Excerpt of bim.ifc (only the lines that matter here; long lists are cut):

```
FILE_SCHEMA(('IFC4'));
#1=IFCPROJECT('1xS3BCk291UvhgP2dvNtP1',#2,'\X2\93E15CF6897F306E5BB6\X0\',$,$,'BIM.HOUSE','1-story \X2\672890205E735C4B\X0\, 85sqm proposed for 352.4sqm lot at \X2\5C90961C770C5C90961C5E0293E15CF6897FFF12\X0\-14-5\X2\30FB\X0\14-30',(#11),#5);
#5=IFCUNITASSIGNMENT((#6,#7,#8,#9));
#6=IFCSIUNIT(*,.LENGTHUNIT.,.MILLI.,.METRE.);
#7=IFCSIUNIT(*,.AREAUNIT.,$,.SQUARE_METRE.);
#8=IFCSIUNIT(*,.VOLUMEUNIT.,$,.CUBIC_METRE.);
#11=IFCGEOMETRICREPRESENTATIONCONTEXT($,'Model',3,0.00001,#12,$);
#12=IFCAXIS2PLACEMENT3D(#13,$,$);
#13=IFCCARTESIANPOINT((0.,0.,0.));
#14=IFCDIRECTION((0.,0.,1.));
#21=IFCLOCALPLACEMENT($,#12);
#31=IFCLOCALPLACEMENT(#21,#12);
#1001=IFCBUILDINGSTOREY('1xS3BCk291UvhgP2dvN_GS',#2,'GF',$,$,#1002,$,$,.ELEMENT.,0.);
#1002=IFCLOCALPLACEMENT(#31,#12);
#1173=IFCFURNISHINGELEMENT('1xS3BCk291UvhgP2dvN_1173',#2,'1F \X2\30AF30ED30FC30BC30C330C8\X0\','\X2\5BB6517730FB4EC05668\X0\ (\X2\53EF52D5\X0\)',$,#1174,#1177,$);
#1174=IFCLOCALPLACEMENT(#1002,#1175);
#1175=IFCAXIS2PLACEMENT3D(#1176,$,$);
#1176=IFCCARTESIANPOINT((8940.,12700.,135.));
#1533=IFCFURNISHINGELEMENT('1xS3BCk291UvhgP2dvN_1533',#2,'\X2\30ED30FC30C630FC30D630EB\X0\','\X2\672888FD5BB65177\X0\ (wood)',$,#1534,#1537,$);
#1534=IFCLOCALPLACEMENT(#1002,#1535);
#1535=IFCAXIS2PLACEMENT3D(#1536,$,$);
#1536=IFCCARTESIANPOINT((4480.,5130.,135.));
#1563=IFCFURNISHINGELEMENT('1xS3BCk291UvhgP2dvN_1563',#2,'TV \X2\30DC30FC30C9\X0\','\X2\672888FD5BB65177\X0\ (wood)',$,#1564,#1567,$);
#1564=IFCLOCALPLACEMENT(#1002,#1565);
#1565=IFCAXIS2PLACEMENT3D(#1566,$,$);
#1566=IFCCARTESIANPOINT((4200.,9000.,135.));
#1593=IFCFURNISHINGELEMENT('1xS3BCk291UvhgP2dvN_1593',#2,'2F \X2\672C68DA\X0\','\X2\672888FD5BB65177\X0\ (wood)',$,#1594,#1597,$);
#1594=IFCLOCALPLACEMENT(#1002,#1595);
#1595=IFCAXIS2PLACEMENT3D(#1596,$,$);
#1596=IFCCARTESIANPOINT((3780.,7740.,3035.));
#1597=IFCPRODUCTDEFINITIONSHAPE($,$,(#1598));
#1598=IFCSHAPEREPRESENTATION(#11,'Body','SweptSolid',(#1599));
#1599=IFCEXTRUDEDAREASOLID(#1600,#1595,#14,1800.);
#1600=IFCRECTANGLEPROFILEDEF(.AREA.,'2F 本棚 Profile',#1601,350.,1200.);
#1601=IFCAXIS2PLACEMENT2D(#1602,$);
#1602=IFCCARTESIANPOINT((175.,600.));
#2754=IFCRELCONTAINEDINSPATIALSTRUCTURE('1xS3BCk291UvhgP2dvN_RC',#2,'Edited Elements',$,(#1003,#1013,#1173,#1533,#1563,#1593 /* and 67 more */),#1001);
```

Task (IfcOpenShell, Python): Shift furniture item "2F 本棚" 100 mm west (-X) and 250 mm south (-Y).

```python
import ifcopenshell
import ifcopenshell.api.geometry
import ifcopenshell.util.placement

model = ifcopenshell.open("bim.ifc")

item = model.by_id(1593)
matrix = ifcopenshell.util.placement.get_local_placement(item.ObjectPlacement)
matrix[0, 3] -= 100.0
matrix[1, 3] -= 250.0
ifcopenshell.api.geometry.edit_object_placement(model, product=item, matrix=matrix, is_si=False)

print(ifcopenshell.util.placement.get_local_placement(item.ObjectPlacement).round(3) + 0.0)

model.write("bim_edited.ifc")
```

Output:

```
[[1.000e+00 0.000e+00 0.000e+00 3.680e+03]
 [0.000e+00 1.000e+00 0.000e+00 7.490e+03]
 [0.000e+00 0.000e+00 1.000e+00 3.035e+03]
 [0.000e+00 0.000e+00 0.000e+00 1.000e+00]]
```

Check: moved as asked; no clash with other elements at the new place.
